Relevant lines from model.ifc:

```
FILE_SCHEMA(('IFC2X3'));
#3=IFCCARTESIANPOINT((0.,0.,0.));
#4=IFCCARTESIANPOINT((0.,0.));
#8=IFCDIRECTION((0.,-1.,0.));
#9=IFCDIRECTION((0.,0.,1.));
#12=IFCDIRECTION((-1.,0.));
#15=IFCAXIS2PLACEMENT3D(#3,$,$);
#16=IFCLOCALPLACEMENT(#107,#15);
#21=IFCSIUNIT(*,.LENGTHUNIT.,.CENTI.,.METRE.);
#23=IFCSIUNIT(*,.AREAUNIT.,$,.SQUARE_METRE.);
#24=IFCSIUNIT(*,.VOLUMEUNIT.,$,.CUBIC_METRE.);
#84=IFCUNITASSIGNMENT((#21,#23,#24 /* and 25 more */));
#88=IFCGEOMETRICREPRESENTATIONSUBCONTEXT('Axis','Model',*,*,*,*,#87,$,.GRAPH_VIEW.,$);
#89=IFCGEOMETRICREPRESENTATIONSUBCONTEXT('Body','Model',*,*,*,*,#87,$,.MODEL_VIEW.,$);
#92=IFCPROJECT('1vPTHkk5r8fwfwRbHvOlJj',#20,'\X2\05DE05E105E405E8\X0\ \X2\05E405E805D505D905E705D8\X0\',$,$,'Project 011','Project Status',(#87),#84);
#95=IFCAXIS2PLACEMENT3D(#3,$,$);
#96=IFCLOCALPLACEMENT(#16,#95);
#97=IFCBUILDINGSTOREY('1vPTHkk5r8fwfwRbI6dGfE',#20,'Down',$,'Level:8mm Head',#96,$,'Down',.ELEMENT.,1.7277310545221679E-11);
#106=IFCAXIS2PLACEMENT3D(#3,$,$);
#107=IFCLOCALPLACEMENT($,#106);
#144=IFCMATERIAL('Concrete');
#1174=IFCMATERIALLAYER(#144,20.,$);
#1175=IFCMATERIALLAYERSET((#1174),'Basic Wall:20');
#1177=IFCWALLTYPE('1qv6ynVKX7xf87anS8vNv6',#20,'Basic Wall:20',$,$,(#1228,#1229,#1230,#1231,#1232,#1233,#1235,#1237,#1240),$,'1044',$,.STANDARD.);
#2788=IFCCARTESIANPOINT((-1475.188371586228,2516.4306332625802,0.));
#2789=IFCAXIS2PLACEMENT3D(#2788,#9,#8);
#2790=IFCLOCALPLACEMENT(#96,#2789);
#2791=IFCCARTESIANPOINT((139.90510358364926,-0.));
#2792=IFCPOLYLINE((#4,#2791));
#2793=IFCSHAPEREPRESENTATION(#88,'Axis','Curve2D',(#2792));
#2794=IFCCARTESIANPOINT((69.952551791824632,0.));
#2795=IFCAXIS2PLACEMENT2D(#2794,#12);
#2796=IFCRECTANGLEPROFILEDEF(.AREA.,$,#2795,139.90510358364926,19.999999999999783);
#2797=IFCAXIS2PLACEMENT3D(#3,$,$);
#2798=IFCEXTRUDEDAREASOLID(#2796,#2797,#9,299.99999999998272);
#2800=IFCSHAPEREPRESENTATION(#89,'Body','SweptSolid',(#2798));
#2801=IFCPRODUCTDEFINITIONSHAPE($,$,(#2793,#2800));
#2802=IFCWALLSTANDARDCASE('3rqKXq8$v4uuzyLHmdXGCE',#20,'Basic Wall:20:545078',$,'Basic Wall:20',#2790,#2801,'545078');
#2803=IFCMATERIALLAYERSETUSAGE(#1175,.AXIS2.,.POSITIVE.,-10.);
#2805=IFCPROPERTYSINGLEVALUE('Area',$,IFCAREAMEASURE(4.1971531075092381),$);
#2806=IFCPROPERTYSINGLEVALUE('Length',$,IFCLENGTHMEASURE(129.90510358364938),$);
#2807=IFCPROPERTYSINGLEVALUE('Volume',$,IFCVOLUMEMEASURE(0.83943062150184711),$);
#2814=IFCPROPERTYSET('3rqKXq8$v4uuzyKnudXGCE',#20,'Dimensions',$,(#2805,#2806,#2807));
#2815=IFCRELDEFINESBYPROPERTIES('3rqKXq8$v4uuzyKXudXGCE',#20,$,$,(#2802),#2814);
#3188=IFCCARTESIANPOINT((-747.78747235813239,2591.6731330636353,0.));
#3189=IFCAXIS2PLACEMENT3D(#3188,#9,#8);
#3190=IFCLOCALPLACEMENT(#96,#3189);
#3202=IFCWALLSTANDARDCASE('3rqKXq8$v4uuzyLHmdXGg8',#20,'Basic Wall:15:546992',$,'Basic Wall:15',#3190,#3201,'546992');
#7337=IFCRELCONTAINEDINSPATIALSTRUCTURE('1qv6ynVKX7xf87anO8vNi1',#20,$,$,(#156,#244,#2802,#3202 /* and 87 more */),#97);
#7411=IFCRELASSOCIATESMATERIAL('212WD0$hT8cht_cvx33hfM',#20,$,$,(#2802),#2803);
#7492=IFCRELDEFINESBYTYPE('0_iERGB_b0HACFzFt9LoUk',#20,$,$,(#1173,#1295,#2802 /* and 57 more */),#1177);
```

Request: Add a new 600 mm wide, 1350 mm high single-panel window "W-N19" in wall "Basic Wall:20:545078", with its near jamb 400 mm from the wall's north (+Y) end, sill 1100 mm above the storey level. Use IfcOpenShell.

```python
import numpy as np
import ifcopenshell
import ifcopenshell.api.feature
import ifcopenshell.api.geometry
import ifcopenshell.api.pset
import ifcopenshell.api.root
import ifcopenshell.api.spatial
import ifcopenshell.api.type
import ifcopenshell.geom
import ifcopenshell.util.element
import ifcopenshell.util.placement
import ifcopenshell.util.representation
import ifcopenshell.util.shape
import ifcopenshell.util.unit

model = ifcopenshell.open("model.ifc")
unit_scale = ifcopenshell.util.unit.calculate_unit_scale(model)
area_scale = ifcopenshell.util.unit.calculate_unit_scale(model, "AREAUNIT")
volume_scale = ifcopenshell.util.unit.calculate_unit_scale(model, "VOLUMEUNIT")
settings = ifcopenshell.geom.settings()


def volume(element):
    """Net volume in cubic metres, openings subtracted."""
    shape = ifcopenshell.geom.create_shape(settings, element)
    return ifcopenshell.util.shape.get_volume(shape.geometry)


wall = model.by_guid("3rqKXq8$v4uuzyLHmdXGCE")
storey = ifcopenshell.util.element.get_container(wall, ifc_class="IfcBuildingStorey")
context = ifcopenshell.util.representation.get_context(model, "Model", "Body", "MODEL_VIEW")
before = volume(wall)

width, height, from_end, sill = 0.6, 1.35, 0.4, 1.1  # metres

# The wall runs along its own X axis, and the end named is its -X end.
wall_shape = ifcopenshell.geom.create_shape(settings, wall)
x, y, z = ifcopenshell.util.shape.get_vertices(wall_shape.geometry).T
start = x.min() + from_end
face, thickness = float(y.min()), float(y.max() - y.min())
wall_matrix = ifcopenshell.util.placement.get_local_placement(wall.ObjectPlacement)
level = ifcopenshell.util.placement.get_local_placement(storey.ObjectPlacement)[2, 3]


def in_wall(x, y):
    """Placement at x, y metres in the wall's axes, at sill height."""
    matrix = wall_matrix.copy()
    matrix[:, 3] = wall_matrix @ np.array([x / unit_scale, y / unit_scale, 0.0, 1.0])
    matrix[2, 3] = level + sill / unit_scale
    return matrix


# Opening: a box that overshoots both wall faces by 50 mm.
opening = ifcopenshell.api.root.create_entity(model, ifc_class="IfcOpeningElement")
box = ifcopenshell.api.geometry.add_wall_representation(
    model, context=context, length=width, height=height, thickness=thickness + 0.1
)
ifcopenshell.api.geometry.assign_representation(model, product=opening, representation=box)
ifcopenshell.api.geometry.edit_object_placement(model, product=opening, matrix=in_wall(start, face - 0.05), is_si=False)
ifcopenshell.api.feature.add_feature(model, feature=opening, element=wall)

window = ifcopenshell.api.root.create_entity(model, ifc_class="IfcWindow", name="W-N19")
window.OverallWidth, window.OverallHeight = width / unit_scale, height / unit_scale
body = ifcopenshell.api.geometry.add_window_representation(
    model,
    context=context,
    overall_width=window.OverallWidth,
    overall_height=window.OverallHeight,
    partition_type="SINGLE_PANEL",
)
ifcopenshell.api.geometry.assign_representation(model, product=window, representation=body)
ifcopenshell.api.spatial.assign_container(model, products=[window], relating_structure=storey)
fills = ifcopenshell.api.feature.add_filling(model, opening=opening, element=window)
fills.OwnerHistory = window.OwnerHistory  # required in IFC2X3

# IFC2X3 keeps the operation on the window style.
style = ifcopenshell.api.root.create_entity(model, ifc_class="IfcWindowStyle", name="W-N19")
style.OperationType, style.ConstructionType = "SINGLE_PANEL", "NOTDEFINED"
style.ParameterTakesPrecedence = style.Sizeable = False
ifcopenshell.api.type.assign_type(model, related_objects=[window], relating_type=style)

# Centre the window in the wall's thickness.
ifcopenshell.api.geometry.edit_object_placement(model, product=window, matrix=in_wall(start, face), is_si=False)
window_shape = ifcopenshell.geom.create_shape(settings, window)
depth = ifcopenshell.util.shape.get_vertices(window_shape.geometry)[:, 1]
offset = face + thickness / 2 - (depth.min() + depth.max()) / 2
ifcopenshell.api.geometry.edit_object_placement(model, product=window, matrix=in_wall(start, offset), is_si=False)

after = volume(wall)

# Update the wall's stored quantities.
pset = model.by_id(ifcopenshell.util.element.get_pset(wall, "Dimensions", should_inherit=False)["id"])
ifcopenshell.api.pset.edit_pset(model, pset=pset, properties={
    "Area": model.create_entity("IfcAreaMeasure", after / thickness / area_scale),
    "Volume": model.create_entity("IfcVolumeMeasure", after / volume_scale),
})

print(f"wall volume {before:.3f} -> {after:.3f} m3")

model.write("model_v2.ifc")
```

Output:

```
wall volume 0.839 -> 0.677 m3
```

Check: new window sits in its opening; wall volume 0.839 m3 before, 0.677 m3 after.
